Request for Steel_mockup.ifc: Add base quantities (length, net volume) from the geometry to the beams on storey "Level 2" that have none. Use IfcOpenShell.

First a look at what the model holds.

```python
import ifcopenshell
import ifcopenshell.util.element
import ifcopenshell.util.unit

model = ifcopenshell.open("Steel_mockup.ifc")
print(model.schema)
for unit_type in ("LENGTHUNIT", "AREAUNIT", "VOLUMEUNIT"):
    print(unit_type, ifcopenshell.util.unit.calculate_unit_scale(model, unit_type))
storey = next(s for s in model.by_type("IfcBuildingStorey") if s.Name == "Level 2")
beams = [e for e in ifcopenshell.util.element.get_decomposition(storey) if e.is_a("IfcBeam")]
for e in sorted(beams, key=lambda e: e.id()):
    print(e.id(), e.is_a(), e.Name, list(ifcopenshell.util.element.get_psets(e, qtos_only=True)), sep=" | ")
```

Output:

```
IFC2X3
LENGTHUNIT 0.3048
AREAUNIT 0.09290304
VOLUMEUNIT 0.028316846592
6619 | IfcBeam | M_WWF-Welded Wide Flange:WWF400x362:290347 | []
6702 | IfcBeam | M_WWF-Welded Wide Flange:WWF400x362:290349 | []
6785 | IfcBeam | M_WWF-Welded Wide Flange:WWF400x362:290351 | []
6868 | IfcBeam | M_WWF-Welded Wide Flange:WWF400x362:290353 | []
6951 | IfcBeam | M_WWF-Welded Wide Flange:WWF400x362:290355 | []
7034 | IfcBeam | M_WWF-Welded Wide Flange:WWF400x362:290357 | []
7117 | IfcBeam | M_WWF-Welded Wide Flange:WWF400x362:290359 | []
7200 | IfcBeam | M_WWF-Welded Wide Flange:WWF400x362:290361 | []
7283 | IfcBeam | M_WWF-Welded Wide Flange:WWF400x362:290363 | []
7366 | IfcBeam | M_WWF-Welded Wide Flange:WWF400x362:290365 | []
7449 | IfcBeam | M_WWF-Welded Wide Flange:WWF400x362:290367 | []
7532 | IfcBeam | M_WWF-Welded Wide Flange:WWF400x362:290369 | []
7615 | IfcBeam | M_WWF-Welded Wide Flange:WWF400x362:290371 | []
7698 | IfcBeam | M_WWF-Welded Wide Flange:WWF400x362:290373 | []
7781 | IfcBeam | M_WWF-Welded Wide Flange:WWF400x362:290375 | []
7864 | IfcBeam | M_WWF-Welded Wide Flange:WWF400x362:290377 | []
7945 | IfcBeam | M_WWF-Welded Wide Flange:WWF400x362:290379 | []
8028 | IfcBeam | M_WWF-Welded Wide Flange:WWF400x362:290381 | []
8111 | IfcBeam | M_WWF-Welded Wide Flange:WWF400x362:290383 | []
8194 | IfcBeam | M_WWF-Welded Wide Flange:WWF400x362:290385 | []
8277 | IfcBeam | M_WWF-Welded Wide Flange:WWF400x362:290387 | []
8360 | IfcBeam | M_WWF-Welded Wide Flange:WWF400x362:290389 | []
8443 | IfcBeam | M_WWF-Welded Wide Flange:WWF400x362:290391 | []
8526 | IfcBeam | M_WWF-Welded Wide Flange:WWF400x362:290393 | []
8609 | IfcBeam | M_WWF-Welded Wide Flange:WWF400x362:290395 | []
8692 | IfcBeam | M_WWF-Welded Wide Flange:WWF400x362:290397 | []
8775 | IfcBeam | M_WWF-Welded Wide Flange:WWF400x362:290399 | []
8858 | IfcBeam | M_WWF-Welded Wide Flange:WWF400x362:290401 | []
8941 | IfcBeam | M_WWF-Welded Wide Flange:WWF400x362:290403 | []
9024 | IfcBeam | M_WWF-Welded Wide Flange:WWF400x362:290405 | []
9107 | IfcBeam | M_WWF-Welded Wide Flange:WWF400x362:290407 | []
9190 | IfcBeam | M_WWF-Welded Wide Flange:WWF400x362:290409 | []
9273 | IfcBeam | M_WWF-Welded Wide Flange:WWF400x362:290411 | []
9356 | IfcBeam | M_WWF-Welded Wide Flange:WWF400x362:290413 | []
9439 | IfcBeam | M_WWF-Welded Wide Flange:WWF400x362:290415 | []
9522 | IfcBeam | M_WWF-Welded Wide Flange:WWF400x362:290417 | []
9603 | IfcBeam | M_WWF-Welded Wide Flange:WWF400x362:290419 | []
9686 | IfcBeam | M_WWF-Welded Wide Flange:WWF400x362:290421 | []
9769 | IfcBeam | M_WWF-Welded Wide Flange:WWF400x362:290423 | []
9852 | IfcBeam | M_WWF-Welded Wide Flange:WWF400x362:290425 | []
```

```python
import ifcopenshell
import ifcopenshell.api.pset
import ifcopenshell.geom
import ifcopenshell.util.element
import ifcopenshell.util.shape
import ifcopenshell.util.unit

model = ifcopenshell.open("Steel_mockup.ifc")
unit_scale = ifcopenshell.util.unit.calculate_unit_scale(model)
volume_scale = ifcopenshell.util.unit.calculate_unit_scale(model, "VOLUMEUNIT")
settings = ifcopenshell.geom.settings()

storey = next(s for s in model.by_type("IfcBuildingStorey") if s.Name == "Level 2")
beams = [e for e in ifcopenshell.util.element.get_decomposition(storey) if e.is_a("IfcBeam")]

for e in sorted(beams, key=lambda e: e.id()):
    if ifcopenshell.util.element.get_psets(e, qtos_only=True, should_inherit=False):
        continue
    # Geometry comes back in metres, in the element's own axes.
    shape = ifcopenshell.geom.create_shape(settings, e)
    values = {
        "Length": ifcopenshell.util.shape.get_max_xyz(shape.geometry) / unit_scale,
        "NetVolume": ifcopenshell.util.shape.get_volume(shape.geometry) / volume_scale,
    }
    qto = ifcopenshell.api.pset.add_qto(model, product=e, name="BaseQuantities")
    ifcopenshell.api.pset.edit_qto(model, qto=qto, properties=values)
    print(e.id(), {k: round(v, 3) for k, v in values.items()})

model.write("Steel_mockup_rev.ifc")
```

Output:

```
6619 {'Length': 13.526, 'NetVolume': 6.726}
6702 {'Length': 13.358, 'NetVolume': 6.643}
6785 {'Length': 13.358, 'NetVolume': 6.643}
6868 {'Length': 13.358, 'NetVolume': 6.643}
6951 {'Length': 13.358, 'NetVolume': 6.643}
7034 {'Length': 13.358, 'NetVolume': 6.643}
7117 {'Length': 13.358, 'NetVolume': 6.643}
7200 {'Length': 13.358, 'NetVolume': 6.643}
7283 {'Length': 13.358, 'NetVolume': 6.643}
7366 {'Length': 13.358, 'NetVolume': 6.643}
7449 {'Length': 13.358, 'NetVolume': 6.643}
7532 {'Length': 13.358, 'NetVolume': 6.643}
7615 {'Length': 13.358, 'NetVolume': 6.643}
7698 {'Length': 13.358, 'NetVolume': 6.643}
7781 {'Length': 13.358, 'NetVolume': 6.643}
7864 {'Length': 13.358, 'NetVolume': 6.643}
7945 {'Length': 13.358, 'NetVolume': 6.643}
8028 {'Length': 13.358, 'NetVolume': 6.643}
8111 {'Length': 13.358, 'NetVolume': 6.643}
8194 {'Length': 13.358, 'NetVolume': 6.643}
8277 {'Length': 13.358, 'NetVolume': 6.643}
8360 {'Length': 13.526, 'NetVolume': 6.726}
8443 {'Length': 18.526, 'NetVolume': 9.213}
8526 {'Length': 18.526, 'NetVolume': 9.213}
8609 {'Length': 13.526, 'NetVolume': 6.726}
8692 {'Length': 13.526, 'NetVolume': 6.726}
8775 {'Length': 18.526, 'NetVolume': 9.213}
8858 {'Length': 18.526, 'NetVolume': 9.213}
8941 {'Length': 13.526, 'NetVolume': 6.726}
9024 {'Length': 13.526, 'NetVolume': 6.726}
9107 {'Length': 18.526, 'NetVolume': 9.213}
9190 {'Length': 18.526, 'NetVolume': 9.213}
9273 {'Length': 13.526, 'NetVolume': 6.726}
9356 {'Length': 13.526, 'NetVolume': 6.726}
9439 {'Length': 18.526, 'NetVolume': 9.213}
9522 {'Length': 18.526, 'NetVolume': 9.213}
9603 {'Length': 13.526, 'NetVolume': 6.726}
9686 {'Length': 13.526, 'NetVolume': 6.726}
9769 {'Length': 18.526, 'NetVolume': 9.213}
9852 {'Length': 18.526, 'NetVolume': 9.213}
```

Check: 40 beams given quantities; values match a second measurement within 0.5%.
